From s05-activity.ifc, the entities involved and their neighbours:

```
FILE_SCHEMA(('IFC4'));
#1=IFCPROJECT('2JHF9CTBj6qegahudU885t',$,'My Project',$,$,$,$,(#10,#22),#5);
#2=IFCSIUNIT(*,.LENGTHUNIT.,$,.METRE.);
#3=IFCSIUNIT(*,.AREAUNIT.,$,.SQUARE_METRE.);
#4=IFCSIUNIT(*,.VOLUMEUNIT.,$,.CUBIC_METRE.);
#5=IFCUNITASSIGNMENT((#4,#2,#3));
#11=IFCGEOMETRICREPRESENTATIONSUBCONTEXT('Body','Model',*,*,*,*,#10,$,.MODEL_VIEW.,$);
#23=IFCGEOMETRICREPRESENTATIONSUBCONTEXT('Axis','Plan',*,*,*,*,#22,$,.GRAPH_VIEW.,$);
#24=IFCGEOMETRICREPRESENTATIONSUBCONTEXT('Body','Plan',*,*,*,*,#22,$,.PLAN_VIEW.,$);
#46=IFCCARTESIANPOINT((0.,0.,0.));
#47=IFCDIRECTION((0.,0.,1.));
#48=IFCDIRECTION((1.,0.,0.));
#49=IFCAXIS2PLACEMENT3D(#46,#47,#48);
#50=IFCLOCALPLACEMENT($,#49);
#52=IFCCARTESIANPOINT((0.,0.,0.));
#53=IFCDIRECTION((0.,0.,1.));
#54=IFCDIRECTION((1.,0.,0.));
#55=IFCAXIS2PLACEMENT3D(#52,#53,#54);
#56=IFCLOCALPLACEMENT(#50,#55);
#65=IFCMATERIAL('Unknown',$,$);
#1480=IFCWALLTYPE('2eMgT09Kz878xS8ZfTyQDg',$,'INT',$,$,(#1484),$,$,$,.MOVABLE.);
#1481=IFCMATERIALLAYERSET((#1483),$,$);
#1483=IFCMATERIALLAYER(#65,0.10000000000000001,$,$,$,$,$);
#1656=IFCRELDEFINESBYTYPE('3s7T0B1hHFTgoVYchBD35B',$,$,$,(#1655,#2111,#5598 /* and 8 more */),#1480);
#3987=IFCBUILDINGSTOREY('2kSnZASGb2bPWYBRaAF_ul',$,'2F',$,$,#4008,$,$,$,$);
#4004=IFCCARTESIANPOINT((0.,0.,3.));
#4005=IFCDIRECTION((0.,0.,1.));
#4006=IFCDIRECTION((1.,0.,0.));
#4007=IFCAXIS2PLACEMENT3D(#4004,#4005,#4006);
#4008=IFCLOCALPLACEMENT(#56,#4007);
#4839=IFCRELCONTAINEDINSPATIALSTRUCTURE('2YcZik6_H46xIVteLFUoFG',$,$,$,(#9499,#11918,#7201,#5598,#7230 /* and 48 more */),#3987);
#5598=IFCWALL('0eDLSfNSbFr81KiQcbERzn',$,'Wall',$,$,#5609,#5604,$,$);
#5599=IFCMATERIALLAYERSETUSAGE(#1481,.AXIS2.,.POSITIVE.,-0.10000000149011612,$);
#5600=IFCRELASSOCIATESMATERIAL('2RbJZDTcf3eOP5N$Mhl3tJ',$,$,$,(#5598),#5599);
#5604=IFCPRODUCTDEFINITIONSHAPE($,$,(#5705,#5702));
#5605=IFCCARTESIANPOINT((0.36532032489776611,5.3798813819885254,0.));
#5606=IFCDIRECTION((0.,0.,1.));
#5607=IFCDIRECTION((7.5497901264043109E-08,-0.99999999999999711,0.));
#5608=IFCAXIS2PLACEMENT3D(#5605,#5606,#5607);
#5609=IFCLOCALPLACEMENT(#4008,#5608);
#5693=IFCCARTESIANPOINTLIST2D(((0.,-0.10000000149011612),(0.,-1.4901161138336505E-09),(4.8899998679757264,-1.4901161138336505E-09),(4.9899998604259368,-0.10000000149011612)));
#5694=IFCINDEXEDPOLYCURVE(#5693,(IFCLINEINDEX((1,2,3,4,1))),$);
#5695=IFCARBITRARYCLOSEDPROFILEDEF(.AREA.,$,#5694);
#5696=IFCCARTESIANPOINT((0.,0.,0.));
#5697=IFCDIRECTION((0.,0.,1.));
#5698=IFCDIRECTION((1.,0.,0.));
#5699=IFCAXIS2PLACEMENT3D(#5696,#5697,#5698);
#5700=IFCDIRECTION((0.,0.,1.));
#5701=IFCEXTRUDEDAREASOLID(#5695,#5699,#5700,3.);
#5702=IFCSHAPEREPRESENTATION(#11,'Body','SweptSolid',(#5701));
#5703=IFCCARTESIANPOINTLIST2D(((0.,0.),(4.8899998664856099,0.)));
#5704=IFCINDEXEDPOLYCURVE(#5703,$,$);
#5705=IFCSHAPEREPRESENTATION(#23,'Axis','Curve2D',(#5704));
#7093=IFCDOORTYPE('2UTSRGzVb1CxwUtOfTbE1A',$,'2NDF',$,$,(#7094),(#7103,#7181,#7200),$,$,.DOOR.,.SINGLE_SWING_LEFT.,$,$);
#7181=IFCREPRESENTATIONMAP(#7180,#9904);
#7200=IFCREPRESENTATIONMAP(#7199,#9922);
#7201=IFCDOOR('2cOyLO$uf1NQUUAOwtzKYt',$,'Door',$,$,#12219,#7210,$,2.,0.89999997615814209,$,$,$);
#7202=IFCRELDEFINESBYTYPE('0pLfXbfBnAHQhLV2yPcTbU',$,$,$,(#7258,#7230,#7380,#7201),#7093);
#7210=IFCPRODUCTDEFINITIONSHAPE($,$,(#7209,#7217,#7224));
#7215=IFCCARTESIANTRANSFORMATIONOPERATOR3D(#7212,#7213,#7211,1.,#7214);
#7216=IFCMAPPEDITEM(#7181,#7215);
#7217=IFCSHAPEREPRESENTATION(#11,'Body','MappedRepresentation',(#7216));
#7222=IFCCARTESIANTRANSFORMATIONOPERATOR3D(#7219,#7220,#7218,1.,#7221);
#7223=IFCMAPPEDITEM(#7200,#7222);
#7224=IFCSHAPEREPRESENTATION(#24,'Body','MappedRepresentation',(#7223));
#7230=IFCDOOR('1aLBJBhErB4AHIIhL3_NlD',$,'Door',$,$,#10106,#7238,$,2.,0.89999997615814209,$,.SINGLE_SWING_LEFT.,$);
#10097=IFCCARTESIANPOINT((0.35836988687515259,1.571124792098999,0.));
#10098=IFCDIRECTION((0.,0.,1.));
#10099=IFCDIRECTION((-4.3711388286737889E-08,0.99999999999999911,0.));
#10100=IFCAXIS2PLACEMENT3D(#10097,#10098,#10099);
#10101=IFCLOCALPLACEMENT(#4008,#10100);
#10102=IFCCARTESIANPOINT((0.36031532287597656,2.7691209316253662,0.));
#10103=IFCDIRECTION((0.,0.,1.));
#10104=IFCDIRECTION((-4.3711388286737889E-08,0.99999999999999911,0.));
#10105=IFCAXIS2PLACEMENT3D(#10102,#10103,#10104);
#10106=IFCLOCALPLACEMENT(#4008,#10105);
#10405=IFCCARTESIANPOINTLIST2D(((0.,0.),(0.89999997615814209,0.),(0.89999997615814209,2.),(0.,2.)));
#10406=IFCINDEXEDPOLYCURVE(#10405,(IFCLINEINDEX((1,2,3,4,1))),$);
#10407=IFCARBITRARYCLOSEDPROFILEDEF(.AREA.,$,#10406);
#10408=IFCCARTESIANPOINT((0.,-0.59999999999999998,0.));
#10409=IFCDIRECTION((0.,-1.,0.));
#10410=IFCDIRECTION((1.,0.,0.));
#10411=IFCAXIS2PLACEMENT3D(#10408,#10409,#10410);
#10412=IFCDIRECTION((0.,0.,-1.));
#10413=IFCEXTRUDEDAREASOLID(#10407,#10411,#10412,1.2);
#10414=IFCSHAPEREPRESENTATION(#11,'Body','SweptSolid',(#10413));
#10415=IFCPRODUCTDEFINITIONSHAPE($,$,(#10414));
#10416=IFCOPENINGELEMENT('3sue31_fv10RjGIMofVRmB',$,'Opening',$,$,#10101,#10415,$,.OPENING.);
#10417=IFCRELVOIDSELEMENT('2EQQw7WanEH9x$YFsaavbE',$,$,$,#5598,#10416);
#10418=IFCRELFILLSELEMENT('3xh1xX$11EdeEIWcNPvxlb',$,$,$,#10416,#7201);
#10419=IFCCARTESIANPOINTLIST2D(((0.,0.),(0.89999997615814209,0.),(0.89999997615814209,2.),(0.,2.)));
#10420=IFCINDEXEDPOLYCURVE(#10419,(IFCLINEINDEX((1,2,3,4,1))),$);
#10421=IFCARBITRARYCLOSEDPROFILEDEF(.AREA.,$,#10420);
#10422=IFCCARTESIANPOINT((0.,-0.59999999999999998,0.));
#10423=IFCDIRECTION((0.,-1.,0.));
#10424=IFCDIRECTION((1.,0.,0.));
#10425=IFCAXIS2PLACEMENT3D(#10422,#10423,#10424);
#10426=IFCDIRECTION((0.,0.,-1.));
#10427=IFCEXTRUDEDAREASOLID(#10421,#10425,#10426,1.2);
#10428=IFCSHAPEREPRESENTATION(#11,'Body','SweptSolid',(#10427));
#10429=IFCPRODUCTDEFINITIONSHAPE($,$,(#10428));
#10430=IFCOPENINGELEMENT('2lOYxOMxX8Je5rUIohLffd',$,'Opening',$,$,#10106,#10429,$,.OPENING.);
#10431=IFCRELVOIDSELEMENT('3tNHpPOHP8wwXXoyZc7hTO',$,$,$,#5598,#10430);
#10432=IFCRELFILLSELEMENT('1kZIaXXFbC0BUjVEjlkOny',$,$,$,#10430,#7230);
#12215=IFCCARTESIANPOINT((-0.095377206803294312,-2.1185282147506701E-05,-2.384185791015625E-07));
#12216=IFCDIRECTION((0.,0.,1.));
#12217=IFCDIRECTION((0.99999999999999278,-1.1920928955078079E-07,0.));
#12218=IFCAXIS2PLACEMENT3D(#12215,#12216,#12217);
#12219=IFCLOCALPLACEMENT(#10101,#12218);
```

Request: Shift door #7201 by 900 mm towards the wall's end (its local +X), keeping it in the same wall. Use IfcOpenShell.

```python
import ifcopenshell
import ifcopenshell.api.geometry
import ifcopenshell.util.placement
import ifcopenshell.util.unit

model = ifcopenshell.open("s05-activity.ifc")
unit_scale = ifcopenshell.util.unit.calculate_unit_scale(model)

door = model.by_guid("2cOyLO$uf1NQUUAOwtzKYt")
opening = door.FillsVoids[0].RelatingOpeningElement
wall = opening.VoidsElements[0].RelatingBuildingElement

wall_matrix = ifcopenshell.util.placement.get_local_placement(wall.ObjectPlacement)
shift = wall_matrix[:3, 0] * 0.9 / unit_scale
before = ifcopenshell.util.placement.get_local_placement(door.ObjectPlacement)[:3, 3].copy()

# The door is placed relative to its opening, so it follows when the opening moves.
matrix = ifcopenshell.util.placement.get_local_placement(opening.ObjectPlacement)
matrix[:3, 3] += shift
ifcopenshell.api.geometry.edit_object_placement(
    model, product=opening, matrix=matrix, is_si=False, should_transform_children=True
)

after = ifcopenshell.util.placement.get_local_placement(door.ObjectPlacement)[:3, 3]
print("door moved by", (after - before).round(3) + 0.0)

model.write("s05-activity_edited.ifc")
```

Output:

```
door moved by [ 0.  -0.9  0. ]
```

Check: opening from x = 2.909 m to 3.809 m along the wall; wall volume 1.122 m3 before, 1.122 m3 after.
